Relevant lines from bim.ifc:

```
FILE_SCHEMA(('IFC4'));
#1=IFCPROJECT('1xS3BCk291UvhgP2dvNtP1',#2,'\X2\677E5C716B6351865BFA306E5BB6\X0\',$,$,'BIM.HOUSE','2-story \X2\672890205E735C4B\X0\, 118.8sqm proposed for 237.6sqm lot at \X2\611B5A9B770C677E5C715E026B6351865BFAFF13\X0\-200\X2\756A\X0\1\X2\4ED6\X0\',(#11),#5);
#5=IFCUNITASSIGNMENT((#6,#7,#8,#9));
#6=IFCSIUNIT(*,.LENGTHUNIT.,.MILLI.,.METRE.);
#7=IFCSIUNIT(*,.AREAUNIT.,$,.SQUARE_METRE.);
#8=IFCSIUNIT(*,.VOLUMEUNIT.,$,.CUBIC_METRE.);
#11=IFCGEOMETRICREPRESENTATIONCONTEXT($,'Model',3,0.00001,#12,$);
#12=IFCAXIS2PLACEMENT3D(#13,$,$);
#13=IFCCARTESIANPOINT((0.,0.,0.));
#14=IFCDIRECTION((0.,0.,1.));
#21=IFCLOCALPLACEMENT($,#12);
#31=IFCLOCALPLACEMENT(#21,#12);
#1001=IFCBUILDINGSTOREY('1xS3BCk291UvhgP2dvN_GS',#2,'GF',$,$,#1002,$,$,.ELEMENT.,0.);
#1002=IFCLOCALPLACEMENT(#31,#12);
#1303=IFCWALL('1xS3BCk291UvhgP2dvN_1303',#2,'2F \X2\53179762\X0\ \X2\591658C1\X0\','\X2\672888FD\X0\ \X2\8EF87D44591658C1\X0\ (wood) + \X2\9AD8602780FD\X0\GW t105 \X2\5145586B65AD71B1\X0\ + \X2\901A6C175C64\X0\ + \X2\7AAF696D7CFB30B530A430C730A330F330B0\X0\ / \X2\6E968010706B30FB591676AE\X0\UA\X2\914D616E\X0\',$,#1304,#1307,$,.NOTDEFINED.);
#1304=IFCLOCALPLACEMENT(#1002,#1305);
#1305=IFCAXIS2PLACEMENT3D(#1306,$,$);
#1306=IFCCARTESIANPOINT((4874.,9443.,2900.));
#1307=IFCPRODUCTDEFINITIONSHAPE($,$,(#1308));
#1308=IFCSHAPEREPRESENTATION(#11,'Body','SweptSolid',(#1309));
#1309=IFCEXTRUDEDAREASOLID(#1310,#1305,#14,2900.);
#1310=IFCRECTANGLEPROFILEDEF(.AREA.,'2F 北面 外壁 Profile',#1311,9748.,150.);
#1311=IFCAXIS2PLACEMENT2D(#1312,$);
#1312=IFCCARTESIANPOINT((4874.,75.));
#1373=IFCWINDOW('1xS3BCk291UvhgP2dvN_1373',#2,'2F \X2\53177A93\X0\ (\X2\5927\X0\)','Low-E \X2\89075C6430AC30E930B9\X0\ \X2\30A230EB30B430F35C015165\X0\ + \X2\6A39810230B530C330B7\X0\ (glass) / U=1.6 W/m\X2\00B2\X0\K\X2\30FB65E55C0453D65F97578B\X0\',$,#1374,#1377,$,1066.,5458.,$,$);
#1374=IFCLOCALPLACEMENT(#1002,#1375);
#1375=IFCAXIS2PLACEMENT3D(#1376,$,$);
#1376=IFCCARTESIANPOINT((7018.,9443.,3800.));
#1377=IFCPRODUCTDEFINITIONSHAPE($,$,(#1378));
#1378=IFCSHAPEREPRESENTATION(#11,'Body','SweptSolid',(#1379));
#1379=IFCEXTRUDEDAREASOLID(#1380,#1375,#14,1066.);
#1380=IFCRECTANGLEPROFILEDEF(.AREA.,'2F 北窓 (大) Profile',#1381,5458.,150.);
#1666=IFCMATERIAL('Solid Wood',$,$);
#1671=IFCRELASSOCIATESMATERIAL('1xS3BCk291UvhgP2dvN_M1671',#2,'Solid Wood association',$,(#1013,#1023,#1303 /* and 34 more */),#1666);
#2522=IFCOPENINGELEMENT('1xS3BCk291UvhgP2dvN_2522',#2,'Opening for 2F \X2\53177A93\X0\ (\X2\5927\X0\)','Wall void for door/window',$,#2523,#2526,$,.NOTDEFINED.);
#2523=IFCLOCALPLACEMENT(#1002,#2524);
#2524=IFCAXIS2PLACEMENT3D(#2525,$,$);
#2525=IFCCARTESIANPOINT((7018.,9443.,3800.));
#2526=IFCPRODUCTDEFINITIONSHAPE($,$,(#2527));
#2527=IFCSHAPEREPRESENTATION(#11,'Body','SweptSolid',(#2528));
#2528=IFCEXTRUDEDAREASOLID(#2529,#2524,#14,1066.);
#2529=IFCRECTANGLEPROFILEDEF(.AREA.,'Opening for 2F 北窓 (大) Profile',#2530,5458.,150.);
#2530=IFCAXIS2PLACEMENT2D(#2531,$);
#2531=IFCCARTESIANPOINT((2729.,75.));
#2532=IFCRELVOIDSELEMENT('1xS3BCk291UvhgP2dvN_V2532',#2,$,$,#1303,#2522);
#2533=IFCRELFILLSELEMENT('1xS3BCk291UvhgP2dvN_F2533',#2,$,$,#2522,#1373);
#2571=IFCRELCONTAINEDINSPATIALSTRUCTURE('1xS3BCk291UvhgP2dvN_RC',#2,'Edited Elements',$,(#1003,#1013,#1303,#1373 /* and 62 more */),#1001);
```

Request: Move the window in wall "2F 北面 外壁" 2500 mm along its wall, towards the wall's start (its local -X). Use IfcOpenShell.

```python
import ifcopenshell
import ifcopenshell.api.geometry
import ifcopenshell.util.placement

model = ifcopenshell.open("bim.ifc")

window = model.by_guid("1xS3BCk291UvhgP2dvN_1373")
opening = window.FillsVoids[0].RelatingOpeningElement
wall = opening.VoidsElements[0].RelatingBuildingElement

wall_matrix = ifcopenshell.util.placement.get_local_placement(wall.ObjectPlacement)
shift = wall_matrix[:3, 0] * -2500.0
before = ifcopenshell.util.placement.get_local_placement(window.ObjectPlacement)[:3, 3].copy()

# The window is not placed relative to its opening, so move both.
for product in (opening, window):
    matrix = ifcopenshell.util.placement.get_local_placement(product.ObjectPlacement)
    matrix[:3, 3] += shift
    ifcopenshell.api.geometry.edit_object_placement(model, product=product, matrix=matrix, is_si=False)

after = ifcopenshell.util.placement.get_local_placement(window.ObjectPlacement)[:3, 3]
print("window moved by", (after - before).round(3) + 0.0)

model.write("bim_edited.ifc")
```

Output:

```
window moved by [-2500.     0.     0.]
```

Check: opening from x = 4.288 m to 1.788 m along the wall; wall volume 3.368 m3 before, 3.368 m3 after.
